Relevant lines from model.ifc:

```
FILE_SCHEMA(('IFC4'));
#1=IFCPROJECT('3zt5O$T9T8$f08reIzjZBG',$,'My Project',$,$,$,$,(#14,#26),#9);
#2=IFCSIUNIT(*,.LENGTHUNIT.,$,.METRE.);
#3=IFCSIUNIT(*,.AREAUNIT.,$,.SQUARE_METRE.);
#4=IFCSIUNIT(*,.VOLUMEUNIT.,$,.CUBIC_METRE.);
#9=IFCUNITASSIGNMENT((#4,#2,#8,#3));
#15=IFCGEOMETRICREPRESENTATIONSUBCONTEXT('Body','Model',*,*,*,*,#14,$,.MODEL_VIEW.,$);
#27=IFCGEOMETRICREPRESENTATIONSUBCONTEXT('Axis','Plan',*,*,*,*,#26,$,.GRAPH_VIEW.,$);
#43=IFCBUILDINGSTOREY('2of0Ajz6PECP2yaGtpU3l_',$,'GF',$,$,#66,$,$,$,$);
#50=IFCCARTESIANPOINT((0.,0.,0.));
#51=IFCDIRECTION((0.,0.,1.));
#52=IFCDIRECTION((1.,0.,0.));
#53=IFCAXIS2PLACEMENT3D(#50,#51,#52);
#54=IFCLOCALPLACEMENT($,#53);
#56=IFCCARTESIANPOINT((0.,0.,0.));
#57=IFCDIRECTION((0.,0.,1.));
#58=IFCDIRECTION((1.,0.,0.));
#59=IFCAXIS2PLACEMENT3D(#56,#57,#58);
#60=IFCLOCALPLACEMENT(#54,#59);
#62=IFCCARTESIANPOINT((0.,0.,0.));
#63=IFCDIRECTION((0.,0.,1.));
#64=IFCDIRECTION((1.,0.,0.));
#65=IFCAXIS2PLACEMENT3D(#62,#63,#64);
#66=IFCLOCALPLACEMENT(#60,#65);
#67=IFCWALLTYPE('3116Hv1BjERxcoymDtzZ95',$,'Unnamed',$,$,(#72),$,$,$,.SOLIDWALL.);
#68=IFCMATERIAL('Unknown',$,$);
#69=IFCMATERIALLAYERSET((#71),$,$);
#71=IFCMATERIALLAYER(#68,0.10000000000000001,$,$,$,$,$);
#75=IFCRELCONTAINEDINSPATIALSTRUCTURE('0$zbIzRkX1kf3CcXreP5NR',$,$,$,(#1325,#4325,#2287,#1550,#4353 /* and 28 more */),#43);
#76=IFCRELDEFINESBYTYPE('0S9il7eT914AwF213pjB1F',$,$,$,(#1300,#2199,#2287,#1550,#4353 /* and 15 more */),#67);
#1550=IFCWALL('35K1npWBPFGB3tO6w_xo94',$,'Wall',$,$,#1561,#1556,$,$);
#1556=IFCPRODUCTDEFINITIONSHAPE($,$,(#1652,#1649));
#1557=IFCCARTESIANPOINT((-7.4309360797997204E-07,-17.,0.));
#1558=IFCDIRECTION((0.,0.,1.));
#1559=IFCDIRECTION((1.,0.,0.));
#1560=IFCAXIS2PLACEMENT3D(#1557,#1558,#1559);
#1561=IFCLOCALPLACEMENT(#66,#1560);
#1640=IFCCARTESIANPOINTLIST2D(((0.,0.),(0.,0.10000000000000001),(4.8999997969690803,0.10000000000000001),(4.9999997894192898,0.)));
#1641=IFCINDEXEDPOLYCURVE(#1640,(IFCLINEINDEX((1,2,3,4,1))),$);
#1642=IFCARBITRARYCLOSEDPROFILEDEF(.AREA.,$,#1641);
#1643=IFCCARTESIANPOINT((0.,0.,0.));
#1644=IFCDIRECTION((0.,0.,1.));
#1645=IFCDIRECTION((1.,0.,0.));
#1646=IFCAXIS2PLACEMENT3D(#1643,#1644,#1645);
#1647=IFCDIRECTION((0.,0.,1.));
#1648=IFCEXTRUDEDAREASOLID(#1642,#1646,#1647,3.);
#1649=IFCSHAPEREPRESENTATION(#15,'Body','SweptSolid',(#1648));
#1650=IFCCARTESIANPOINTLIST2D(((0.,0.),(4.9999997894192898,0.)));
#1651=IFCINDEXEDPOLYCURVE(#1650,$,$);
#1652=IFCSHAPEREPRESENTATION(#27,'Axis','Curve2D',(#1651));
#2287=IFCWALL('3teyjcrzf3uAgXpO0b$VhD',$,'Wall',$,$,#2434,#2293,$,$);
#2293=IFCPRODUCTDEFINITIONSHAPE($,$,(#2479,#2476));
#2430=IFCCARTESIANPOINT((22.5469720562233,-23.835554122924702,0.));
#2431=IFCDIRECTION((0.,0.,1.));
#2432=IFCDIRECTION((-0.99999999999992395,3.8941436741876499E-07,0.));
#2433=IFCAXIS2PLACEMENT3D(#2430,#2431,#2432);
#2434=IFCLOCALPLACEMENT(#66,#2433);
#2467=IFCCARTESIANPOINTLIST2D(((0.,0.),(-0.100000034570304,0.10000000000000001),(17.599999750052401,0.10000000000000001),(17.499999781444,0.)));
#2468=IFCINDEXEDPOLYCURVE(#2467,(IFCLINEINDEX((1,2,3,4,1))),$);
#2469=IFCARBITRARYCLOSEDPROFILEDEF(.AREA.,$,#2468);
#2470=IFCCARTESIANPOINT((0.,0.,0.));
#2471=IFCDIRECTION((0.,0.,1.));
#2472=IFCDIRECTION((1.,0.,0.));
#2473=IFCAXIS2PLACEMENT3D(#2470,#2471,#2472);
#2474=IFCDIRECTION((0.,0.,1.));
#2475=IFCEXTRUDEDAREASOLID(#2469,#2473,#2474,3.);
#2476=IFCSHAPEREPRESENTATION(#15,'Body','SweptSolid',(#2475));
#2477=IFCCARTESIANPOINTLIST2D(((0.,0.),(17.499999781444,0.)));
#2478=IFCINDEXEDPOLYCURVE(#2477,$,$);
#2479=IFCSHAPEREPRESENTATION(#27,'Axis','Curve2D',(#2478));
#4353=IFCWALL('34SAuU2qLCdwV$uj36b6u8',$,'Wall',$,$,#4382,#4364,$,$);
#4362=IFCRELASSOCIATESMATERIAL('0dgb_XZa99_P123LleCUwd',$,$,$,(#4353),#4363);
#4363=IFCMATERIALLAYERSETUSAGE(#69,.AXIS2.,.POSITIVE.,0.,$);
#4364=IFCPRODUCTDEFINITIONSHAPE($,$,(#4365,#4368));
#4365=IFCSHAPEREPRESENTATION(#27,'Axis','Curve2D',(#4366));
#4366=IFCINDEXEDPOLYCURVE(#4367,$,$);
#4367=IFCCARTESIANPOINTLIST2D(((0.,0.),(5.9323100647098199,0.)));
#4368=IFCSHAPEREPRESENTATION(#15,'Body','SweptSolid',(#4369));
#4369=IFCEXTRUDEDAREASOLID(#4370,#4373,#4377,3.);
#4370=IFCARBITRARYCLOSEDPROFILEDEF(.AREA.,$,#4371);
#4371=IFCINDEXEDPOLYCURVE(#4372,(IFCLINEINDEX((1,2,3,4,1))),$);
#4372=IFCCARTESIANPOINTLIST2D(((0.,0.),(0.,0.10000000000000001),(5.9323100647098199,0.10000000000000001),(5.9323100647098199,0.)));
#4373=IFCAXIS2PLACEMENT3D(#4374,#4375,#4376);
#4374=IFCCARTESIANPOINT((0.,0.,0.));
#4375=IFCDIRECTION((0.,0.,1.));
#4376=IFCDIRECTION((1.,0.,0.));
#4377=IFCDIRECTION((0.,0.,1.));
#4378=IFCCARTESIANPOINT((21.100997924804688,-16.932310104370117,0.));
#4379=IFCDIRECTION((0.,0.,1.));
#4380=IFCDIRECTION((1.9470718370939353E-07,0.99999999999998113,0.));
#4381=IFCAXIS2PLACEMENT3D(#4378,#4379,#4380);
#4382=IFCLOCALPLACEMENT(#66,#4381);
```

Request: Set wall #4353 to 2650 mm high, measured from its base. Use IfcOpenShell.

```python
import ifcopenshell
import ifcopenshell.geom
import ifcopenshell.util.representation
import ifcopenshell.util.shape
import ifcopenshell.util.unit

model = ifcopenshell.open("model.ifc")
unit_scale = ifcopenshell.util.unit.calculate_unit_scale(model)
settings = ifcopenshell.geom.settings()


def volume(element):
    """Net volume in cubic metres, openings subtracted."""
    shape = ifcopenshell.geom.create_shape(settings, element)
    return ifcopenshell.util.shape.get_volume(shape.geometry)


wall = model.by_guid("34SAuU2qLCdwV$uj36b6u8")
before = volume(wall)

body = ifcopenshell.util.representation.get_representation(wall, "Model", "Body")
solid = body.Items[0]
old_height = solid.Depth
solid.Depth = 2.65 / unit_scale
after = volume(wall)

print(f"height {old_height:g} -> {solid.Depth:g}, volume {before:.3f} -> {after:.3f} m3")

model.write("model_updated.ifc")
```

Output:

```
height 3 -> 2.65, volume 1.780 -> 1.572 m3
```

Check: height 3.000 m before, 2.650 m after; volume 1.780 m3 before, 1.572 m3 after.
